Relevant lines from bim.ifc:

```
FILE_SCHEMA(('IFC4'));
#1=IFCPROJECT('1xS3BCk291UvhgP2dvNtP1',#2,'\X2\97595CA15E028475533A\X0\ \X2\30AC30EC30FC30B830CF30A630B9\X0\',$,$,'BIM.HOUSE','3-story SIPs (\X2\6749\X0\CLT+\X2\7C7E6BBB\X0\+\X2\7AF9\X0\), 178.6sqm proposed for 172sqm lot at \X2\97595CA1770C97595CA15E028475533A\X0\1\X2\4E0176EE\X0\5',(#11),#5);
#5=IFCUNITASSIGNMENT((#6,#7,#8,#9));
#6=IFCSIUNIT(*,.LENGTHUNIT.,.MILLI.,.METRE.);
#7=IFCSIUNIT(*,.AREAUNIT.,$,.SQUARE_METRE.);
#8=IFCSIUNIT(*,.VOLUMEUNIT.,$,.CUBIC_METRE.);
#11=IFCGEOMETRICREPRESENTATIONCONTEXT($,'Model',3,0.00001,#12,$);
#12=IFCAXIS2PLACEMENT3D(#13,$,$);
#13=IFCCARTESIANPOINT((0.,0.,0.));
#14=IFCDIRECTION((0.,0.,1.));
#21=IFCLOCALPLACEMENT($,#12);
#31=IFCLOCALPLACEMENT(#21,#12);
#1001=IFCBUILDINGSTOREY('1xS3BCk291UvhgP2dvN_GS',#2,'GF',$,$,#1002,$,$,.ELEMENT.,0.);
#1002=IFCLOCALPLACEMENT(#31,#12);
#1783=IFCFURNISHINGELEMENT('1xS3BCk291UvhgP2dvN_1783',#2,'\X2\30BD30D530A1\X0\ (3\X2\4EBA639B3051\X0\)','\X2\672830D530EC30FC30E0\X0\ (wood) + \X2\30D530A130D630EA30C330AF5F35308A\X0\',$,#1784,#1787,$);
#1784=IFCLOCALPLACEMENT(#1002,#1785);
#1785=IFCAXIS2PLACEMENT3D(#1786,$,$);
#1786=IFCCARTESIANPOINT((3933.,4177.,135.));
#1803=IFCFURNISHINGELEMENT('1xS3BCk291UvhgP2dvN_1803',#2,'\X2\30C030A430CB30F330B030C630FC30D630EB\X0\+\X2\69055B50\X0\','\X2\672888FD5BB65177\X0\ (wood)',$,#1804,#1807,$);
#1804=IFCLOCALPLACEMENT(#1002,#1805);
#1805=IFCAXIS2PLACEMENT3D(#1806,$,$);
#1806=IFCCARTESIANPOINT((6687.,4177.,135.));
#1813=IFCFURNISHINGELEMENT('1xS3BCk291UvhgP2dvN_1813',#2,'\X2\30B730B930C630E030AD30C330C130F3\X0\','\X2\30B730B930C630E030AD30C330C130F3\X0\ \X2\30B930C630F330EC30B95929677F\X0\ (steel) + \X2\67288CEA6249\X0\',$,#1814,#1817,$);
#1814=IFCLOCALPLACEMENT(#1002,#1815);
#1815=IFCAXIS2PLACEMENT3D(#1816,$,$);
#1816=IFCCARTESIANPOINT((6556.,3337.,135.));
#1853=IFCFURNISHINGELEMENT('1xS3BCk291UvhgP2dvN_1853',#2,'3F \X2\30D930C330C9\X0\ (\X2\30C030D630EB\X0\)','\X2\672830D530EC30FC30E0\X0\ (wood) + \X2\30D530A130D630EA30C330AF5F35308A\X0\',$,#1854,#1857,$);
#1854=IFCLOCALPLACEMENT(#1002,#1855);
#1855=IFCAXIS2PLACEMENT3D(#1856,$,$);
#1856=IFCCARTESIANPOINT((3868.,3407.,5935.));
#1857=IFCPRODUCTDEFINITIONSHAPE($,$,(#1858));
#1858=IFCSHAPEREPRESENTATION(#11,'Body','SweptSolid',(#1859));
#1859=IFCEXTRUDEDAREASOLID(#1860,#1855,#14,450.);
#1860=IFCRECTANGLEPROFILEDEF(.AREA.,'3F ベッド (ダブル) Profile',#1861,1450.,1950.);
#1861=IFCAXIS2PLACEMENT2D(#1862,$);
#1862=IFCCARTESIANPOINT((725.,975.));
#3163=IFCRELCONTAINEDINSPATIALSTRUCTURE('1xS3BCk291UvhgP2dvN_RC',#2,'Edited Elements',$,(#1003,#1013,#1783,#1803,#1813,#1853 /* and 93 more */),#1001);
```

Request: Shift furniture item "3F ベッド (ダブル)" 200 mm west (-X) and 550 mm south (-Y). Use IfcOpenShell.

```python
import ifcopenshell
import ifcopenshell.api.geometry
import ifcopenshell.util.placement

model = ifcopenshell.open("bim.ifc")

item = model.by_guid("1xS3BCk291UvhgP2dvN_1853")
matrix = ifcopenshell.util.placement.get_local_placement(item.ObjectPlacement)
matrix[0, 3] -= 200.0
matrix[1, 3] -= 550.0
ifcopenshell.api.geometry.edit_object_placement(model, product=item, matrix=matrix, is_si=False)

print(ifcopenshell.util.placement.get_local_placement(item.ObjectPlacement).round(3) + 0.0)

model.write("bim_updated.ifc")
```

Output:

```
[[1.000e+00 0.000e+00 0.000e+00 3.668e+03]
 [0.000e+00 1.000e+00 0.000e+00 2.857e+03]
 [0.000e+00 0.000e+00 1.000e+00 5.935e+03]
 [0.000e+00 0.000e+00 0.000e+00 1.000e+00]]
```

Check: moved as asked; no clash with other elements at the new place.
